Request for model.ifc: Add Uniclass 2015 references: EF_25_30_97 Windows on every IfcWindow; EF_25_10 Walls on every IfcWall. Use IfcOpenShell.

First a look at what the model holds.

```python
import ifcopenshell

model = ifcopenshell.open("model.ifc")
print(model.schema)
print("classifications:", [c.Name for c in model.by_type("IfcClassification")])
for ifc_class in ("IfcDoor", "IfcRoof", "IfcStair", "IfcWall", "IfcWindow"):
    print(ifc_class, len(model.by_type(ifc_class)))
```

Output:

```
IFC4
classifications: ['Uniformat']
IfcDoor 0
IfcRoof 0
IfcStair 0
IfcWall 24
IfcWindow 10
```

```python
import ifcopenshell
import ifcopenshell.api.classification

model = ifcopenshell.open("model.ifc")

system = ifcopenshell.api.classification.add_classification(model, classification="Uniclass 2015")

codes = {
    "IfcWindow": ("EF_25_30_97", "Windows"),
    "IfcWall": ("EF_25_10", "Walls"),
}
for ifc_class, (code, name) in codes.items():
    products = model.by_type(ifc_class)
    ifcopenshell.api.classification.add_reference(
        model, products=products, classification=system, identification=code, name=name
    )
    print(code, len(products))

model.write("model_rev.ifc")
```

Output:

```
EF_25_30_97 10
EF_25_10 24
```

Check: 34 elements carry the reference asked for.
